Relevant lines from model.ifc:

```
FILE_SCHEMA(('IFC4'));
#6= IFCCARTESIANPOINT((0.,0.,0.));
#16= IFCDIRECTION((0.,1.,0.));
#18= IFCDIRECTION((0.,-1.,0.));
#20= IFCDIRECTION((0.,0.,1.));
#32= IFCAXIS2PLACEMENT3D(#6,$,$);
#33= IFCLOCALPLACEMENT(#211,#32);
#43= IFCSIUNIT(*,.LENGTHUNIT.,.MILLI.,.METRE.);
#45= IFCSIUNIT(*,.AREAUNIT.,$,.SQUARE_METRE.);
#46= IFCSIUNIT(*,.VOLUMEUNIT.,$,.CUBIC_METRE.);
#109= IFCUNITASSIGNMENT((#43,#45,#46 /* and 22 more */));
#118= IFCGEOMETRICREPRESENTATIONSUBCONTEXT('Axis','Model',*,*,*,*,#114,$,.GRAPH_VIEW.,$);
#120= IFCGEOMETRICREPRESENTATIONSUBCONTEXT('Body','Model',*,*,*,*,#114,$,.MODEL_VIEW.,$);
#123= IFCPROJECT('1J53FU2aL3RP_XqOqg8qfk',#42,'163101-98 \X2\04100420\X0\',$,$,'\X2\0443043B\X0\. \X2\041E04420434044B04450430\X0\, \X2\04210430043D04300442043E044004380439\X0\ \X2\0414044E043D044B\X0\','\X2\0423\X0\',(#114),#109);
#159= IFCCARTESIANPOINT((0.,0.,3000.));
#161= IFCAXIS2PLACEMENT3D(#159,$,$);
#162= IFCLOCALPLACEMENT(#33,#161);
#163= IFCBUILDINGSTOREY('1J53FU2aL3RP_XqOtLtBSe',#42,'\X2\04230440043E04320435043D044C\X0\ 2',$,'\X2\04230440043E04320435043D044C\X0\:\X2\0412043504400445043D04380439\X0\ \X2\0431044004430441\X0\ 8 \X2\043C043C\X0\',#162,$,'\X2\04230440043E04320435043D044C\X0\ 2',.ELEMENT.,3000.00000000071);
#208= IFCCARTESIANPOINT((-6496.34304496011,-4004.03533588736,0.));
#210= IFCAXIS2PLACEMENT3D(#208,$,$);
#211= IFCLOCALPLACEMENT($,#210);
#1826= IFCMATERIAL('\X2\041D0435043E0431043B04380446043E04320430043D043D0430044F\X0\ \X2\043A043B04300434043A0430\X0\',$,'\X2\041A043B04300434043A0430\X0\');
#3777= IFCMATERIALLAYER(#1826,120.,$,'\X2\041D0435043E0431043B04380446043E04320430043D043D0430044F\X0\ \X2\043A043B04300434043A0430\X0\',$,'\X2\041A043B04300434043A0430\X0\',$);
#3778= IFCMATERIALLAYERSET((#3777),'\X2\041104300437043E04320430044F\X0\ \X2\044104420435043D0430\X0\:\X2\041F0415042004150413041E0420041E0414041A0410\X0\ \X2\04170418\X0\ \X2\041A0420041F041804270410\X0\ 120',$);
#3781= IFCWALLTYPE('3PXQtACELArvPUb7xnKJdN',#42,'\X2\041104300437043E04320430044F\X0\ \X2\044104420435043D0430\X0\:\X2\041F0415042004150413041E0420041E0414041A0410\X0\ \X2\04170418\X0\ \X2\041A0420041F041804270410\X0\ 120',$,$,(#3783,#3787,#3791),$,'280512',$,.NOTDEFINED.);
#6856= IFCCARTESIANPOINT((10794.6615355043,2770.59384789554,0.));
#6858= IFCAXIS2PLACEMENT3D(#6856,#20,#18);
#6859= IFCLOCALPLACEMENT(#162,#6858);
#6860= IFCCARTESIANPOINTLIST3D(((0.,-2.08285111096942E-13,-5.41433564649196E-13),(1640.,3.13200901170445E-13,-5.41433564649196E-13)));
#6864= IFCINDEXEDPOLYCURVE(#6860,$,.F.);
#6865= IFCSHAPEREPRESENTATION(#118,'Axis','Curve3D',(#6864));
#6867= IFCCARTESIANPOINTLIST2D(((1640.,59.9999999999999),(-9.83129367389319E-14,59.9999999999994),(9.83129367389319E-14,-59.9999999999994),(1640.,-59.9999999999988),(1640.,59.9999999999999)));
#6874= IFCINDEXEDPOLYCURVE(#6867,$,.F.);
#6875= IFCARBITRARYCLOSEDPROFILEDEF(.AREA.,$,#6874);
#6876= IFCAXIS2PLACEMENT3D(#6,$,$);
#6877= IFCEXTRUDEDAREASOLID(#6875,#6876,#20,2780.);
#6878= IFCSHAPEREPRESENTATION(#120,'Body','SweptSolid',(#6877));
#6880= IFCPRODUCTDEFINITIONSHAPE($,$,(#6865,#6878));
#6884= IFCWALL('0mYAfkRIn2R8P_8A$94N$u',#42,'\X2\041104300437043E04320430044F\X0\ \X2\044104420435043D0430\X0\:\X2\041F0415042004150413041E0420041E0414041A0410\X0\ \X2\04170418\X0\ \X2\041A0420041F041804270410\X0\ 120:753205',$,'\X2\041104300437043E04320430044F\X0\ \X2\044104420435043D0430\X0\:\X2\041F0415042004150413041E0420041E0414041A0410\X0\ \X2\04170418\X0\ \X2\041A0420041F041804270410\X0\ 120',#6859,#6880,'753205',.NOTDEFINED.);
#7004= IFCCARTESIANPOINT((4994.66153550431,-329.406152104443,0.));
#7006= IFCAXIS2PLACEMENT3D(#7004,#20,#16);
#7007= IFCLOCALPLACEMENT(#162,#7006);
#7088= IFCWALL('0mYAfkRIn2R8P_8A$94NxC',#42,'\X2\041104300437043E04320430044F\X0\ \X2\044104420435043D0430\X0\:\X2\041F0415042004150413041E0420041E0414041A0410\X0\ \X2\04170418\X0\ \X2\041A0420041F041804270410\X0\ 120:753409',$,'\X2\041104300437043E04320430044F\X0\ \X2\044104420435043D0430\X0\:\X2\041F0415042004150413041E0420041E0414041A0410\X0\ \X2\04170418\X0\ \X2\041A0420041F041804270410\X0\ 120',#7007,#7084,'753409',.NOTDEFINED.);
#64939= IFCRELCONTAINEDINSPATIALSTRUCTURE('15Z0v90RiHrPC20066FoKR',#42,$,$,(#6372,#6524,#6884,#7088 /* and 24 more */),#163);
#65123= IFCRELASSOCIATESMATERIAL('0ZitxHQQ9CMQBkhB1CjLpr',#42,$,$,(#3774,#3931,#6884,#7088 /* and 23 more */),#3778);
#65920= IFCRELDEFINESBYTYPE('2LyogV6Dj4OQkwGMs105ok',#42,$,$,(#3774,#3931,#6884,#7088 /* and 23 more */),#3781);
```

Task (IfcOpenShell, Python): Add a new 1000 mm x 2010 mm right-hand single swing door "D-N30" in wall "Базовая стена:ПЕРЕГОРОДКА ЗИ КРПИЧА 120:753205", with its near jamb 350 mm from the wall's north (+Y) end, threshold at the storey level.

```python
import numpy as np
import ifcopenshell
import ifcopenshell.api.feature
import ifcopenshell.api.geometry
import ifcopenshell.api.root
import ifcopenshell.api.spatial
import ifcopenshell.geom
import ifcopenshell.util.element
import ifcopenshell.util.placement
import ifcopenshell.util.representation
import ifcopenshell.util.shape
import ifcopenshell.util.unit

model = ifcopenshell.open("model.ifc")
unit_scale = ifcopenshell.util.unit.calculate_unit_scale(model)
settings = ifcopenshell.geom.settings()


def volume(element):
    """Net volume in cubic metres, openings subtracted."""
    shape = ifcopenshell.geom.create_shape(settings, element)
    return ifcopenshell.util.shape.get_volume(shape.geometry)


wall = model.by_guid("0mYAfkRIn2R8P_8A$94N$u")
storey = ifcopenshell.util.element.get_container(wall, ifc_class="IfcBuildingStorey")
context = ifcopenshell.util.representation.get_context(model, "Model", "Body", "MODEL_VIEW")
before = volume(wall)

width, height, from_end, sill = 1, 2.01, 0.35, 0.0  # metres

# The wall runs along its own X axis, and the end named is its -X end.
wall_shape = ifcopenshell.geom.create_shape(settings, wall)
x, y, z = ifcopenshell.util.shape.get_vertices(wall_shape.geometry).T
start = x.min() + from_end
face, thickness = float(y.min()), float(y.max() - y.min())
wall_matrix = ifcopenshell.util.placement.get_local_placement(wall.ObjectPlacement)
level = ifcopenshell.util.placement.get_local_placement(storey.ObjectPlacement)[2, 3]


def in_wall(x, y):
    """Placement at x, y metres in the wall's axes, at sill height."""
    matrix = wall_matrix.copy()
    matrix[:, 3] = wall_matrix @ np.array([x / unit_scale, y / unit_scale, 0.0, 1.0])
    matrix[2, 3] = level + sill / unit_scale
    return matrix


# Opening: a box that overshoots both wall faces by 50 mm.
opening = ifcopenshell.api.root.create_entity(model, ifc_class="IfcOpeningElement", predefined_type="OPENING")
box = ifcopenshell.api.geometry.add_wall_representation(
    model, context=context, length=width, height=height, thickness=thickness + 0.1
)
ifcopenshell.api.geometry.assign_representation(model, product=opening, representation=box)
ifcopenshell.api.geometry.edit_object_placement(model, product=opening, matrix=in_wall(start, face - 0.05), is_si=False)
ifcopenshell.api.feature.add_feature(model, feature=opening, element=wall)

door = ifcopenshell.api.root.create_entity(model, ifc_class="IfcDoor", name="D-N30", predefined_type="DOOR")
door.OverallWidth, door.OverallHeight = width / unit_scale, height / unit_scale
door.OperationType = "SINGLE_SWING_RIGHT"
body = ifcopenshell.api.geometry.add_door_representation(
    model,
    context=context,
    overall_width=door.OverallWidth,
    overall_height=door.OverallHeight,
    operation_type="SINGLE_SWING_RIGHT",
    lining_properties={"LiningDepth": thickness / unit_scale, "ThresholdDepth": thickness / unit_scale},
)
ifcopenshell.api.geometry.assign_representation(model, product=door, representation=body)
ifcopenshell.api.spatial.assign_container(model, products=[door], relating_structure=storey)
ifcopenshell.api.feature.add_filling(model, opening=opening, element=door)

# The lining spans the wall, so the door starts at the wall face.
ifcopenshell.api.geometry.edit_object_placement(model, product=door, matrix=in_wall(start, face), is_si=False)

after = volume(wall)

print(f"wall volume {before:.3f} -> {after:.3f} m3")

model.write("model_edited.ifc")
```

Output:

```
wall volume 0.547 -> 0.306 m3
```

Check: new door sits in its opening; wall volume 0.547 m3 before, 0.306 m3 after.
